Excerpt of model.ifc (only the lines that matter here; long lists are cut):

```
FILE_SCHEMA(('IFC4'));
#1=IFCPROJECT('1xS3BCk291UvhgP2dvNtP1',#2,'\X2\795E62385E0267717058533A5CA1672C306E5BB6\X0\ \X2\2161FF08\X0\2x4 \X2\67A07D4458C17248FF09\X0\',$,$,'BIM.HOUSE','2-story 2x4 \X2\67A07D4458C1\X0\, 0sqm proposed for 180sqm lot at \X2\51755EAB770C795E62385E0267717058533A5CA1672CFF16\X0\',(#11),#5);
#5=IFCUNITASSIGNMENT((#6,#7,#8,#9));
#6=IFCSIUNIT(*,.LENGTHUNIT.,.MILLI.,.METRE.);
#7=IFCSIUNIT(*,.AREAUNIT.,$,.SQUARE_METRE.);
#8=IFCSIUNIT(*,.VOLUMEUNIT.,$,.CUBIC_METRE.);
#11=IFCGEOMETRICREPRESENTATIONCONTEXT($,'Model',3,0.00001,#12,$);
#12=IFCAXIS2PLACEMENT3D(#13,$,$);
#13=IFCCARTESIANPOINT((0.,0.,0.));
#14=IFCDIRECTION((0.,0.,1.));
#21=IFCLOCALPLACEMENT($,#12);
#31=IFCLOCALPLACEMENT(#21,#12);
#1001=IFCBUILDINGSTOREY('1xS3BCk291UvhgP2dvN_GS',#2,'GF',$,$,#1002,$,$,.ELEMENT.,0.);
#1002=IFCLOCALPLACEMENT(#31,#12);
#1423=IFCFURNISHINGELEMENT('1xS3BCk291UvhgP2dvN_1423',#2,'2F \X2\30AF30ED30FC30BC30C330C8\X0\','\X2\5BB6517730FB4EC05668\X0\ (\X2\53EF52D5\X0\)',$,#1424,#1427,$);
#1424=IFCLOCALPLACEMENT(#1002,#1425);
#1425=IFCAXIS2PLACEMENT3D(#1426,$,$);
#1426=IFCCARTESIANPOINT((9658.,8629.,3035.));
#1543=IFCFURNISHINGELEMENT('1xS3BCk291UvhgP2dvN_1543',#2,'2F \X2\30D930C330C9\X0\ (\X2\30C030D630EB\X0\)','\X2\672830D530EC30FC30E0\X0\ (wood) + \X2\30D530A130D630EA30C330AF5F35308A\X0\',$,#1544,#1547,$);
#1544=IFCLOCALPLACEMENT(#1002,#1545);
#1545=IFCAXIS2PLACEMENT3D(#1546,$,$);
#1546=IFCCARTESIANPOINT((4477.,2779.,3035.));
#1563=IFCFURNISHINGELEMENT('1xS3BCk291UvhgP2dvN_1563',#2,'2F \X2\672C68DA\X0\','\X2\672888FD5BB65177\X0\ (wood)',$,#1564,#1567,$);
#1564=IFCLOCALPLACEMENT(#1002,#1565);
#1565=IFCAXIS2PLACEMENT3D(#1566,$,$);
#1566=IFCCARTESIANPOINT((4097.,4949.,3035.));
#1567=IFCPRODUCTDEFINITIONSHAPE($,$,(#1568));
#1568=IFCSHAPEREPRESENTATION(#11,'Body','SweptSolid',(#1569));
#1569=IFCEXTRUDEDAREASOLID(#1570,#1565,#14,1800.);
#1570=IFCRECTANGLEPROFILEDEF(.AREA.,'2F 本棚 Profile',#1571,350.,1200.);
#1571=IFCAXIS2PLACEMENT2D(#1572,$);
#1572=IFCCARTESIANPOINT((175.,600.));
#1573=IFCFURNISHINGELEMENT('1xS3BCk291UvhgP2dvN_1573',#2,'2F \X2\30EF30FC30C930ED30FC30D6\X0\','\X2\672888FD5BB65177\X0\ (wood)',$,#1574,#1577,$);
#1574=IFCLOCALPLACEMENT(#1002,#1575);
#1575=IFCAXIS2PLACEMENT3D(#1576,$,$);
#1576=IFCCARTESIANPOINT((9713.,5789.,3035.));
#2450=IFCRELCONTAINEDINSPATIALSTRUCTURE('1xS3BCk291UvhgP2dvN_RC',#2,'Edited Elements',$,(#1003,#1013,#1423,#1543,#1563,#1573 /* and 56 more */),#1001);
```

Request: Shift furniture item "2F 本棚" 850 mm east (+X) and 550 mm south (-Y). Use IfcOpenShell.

```python
import ifcopenshell
import ifcopenshell.api.geometry
import ifcopenshell.util.placement
import ifcopenshell.util.unit

model = ifcopenshell.open("model.ifc")
unit_scale = ifcopenshell.util.unit.calculate_unit_scale(model)

item = model.by_id(1563)
matrix = ifcopenshell.util.placement.get_local_placement(item.ObjectPlacement)
matrix[0, 3] += 0.85 / unit_scale
matrix[1, 3] -= 0.55 / unit_scale
ifcopenshell.api.geometry.edit_object_placement(model, product=item, matrix=matrix, is_si=False)

print(ifcopenshell.util.placement.get_local_placement(item.ObjectPlacement).round(3) + 0.0)

model.write("model-out.ifc")
```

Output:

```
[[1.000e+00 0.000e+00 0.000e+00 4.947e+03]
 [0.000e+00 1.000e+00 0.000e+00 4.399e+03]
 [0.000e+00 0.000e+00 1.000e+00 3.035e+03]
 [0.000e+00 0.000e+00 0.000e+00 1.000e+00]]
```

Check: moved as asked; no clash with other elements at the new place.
